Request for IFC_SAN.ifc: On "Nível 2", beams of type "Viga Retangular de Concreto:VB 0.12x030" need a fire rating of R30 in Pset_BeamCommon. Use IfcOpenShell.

First a look at what the model holds.

```python
import ifcopenshell
import ifcopenshell.util.element

model = ifcopenshell.open("IFC_SAN.ifc")
print(model.schema)
storey = next(s for s in model.by_type("IfcBuildingStorey") if s.Name == "Nível 2")
beams = [e for e in ifcopenshell.util.element.get_decomposition(storey) if e.is_a("IfcBeam")]
seen = {}
for e in beams:
    element_type = ifcopenshell.util.element.get_type(e)
    key = (element_type.Name if element_type != e and element_type else None, ifcopenshell.util.element.get_pset(e, "Pset_BeamCommon", "FireRating"))
    seen[key] = seen.get(key, 0) + 1
for (name, value), count in sorted(seen.items(), key=str):
    print(count, "x", name, "|", value)
```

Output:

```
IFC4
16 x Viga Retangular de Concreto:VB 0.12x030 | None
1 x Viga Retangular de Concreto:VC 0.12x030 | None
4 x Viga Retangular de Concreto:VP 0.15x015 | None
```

```python
import ifcopenshell
import ifcopenshell.api.pset
import ifcopenshell.util.element

model = ifcopenshell.open("IFC_SAN.ifc")

storey = next(s for s in model.by_type("IfcBuildingStorey") if s.Name == "Nível 2")
beams = [e for e in ifcopenshell.util.element.get_decomposition(storey) if e.is_a("IfcBeam")]

count = 0
for e in beams:
    element_type = ifcopenshell.util.element.get_type(e)
    if element_type in (None, e) or element_type.Name != "Viga Retangular de Concreto:VB 0.12x030":
        continue
    # add_pset returns the element's existing set when there is one.
    pset = ifcopenshell.api.pset.add_pset(model, product=e, name="Pset_BeamCommon")
    ifcopenshell.api.pset.edit_pset(model, pset=pset, properties={"FireRating": "R30"})
    count += 1

print(count, "beams updated")

model.write("IFC_SAN_v2.ifc")
```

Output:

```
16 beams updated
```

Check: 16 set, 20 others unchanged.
